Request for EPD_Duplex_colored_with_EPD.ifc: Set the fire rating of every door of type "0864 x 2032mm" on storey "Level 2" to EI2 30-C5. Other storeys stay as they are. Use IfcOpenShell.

First a look at what the model holds.

```python
import ifcopenshell
import ifcopenshell.util.element

model = ifcopenshell.open("EPD_Duplex_colored_with_EPD.ifc")
print(model.schema)
storey = next(s for s in model.by_type("IfcBuildingStorey") if s.Name == "Level 2")
doors = [e for e in ifcopenshell.util.element.get_decomposition(storey) if e.is_a("IfcDoor")]
seen = {}
for e in doors:
    element_type = ifcopenshell.util.element.get_type(e)
    key = (element_type.Name if element_type != e and element_type else None, ifcopenshell.util.element.get_pset(e, "Pset_DoorCommon", "FireRating"))
    seen[key] = seen.get(key, 0) + 1
for (name, value), count in sorted(seen.items(), key=str):
    print(count, "x", name, "|", value)
```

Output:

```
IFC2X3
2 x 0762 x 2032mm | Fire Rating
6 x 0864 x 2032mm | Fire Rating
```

```python
import ifcopenshell
import ifcopenshell.api.pset
import ifcopenshell.util.element

model = ifcopenshell.open("EPD_Duplex_colored_with_EPD.ifc")

storey = next(s for s in model.by_type("IfcBuildingStorey") if s.Name == "Level 2")
doors = [e for e in ifcopenshell.util.element.get_decomposition(storey) if e.is_a("IfcDoor")]

count = 0
for e in doors:
    element_type = ifcopenshell.util.element.get_type(e)
    if element_type in (None, e) or element_type.Name != "0864 x 2032mm":
        continue
    # add_pset returns the element's existing set when there is one.
    pset = ifcopenshell.api.pset.add_pset(model, product=e, name="Pset_DoorCommon")
    ifcopenshell.api.pset.edit_pset(model, pset=pset, properties={"FireRating": "EI2 30-C5"})
    count += 1

print(count, "doors updated")

model.write("EPD_Duplex_colored_with_EPD_v2.ifc")
```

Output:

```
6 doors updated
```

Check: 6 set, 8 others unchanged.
